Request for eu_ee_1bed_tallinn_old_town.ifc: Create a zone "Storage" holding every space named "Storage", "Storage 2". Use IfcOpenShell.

First a look at what the model holds.

```python
import ifcopenshell

model = ifcopenshell.open("eu_ee_1bed_tallinn_old_town.ifc")
print(model.schema)
seen = {}
for space in model.by_type("IfcSpace"):
    seen[space.LongName] = seen.get(space.LongName, 0) + 1
for name, count in sorted(seen.items(), key=str):
    print(count, "x", name)
print("zones:", [z.Name for z in model.by_type("IfcZone")][:20])
```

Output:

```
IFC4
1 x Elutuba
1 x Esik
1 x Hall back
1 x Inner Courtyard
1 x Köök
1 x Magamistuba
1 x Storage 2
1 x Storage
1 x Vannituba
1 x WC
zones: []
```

```python
import ifcopenshell
import ifcopenshell.api.group
import ifcopenshell.api.root

model = ifcopenshell.open("eu_ee_1bed_tallinn_old_town.ifc")

names = {"Storage", "Storage 2"}
spaces = [s for s in model.by_type("IfcSpace") if s.LongName in names]

zone = ifcopenshell.api.root.create_entity(model, ifc_class="IfcZone", name="Storage")
ifcopenshell.api.group.assign_group(model, products=spaces, group=zone)
print(len(spaces), "spaces in", zone.Name)

model.write("eu_ee_1bed_tallinn_old_town_edited.ifc")
```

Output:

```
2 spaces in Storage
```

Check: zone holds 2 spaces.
